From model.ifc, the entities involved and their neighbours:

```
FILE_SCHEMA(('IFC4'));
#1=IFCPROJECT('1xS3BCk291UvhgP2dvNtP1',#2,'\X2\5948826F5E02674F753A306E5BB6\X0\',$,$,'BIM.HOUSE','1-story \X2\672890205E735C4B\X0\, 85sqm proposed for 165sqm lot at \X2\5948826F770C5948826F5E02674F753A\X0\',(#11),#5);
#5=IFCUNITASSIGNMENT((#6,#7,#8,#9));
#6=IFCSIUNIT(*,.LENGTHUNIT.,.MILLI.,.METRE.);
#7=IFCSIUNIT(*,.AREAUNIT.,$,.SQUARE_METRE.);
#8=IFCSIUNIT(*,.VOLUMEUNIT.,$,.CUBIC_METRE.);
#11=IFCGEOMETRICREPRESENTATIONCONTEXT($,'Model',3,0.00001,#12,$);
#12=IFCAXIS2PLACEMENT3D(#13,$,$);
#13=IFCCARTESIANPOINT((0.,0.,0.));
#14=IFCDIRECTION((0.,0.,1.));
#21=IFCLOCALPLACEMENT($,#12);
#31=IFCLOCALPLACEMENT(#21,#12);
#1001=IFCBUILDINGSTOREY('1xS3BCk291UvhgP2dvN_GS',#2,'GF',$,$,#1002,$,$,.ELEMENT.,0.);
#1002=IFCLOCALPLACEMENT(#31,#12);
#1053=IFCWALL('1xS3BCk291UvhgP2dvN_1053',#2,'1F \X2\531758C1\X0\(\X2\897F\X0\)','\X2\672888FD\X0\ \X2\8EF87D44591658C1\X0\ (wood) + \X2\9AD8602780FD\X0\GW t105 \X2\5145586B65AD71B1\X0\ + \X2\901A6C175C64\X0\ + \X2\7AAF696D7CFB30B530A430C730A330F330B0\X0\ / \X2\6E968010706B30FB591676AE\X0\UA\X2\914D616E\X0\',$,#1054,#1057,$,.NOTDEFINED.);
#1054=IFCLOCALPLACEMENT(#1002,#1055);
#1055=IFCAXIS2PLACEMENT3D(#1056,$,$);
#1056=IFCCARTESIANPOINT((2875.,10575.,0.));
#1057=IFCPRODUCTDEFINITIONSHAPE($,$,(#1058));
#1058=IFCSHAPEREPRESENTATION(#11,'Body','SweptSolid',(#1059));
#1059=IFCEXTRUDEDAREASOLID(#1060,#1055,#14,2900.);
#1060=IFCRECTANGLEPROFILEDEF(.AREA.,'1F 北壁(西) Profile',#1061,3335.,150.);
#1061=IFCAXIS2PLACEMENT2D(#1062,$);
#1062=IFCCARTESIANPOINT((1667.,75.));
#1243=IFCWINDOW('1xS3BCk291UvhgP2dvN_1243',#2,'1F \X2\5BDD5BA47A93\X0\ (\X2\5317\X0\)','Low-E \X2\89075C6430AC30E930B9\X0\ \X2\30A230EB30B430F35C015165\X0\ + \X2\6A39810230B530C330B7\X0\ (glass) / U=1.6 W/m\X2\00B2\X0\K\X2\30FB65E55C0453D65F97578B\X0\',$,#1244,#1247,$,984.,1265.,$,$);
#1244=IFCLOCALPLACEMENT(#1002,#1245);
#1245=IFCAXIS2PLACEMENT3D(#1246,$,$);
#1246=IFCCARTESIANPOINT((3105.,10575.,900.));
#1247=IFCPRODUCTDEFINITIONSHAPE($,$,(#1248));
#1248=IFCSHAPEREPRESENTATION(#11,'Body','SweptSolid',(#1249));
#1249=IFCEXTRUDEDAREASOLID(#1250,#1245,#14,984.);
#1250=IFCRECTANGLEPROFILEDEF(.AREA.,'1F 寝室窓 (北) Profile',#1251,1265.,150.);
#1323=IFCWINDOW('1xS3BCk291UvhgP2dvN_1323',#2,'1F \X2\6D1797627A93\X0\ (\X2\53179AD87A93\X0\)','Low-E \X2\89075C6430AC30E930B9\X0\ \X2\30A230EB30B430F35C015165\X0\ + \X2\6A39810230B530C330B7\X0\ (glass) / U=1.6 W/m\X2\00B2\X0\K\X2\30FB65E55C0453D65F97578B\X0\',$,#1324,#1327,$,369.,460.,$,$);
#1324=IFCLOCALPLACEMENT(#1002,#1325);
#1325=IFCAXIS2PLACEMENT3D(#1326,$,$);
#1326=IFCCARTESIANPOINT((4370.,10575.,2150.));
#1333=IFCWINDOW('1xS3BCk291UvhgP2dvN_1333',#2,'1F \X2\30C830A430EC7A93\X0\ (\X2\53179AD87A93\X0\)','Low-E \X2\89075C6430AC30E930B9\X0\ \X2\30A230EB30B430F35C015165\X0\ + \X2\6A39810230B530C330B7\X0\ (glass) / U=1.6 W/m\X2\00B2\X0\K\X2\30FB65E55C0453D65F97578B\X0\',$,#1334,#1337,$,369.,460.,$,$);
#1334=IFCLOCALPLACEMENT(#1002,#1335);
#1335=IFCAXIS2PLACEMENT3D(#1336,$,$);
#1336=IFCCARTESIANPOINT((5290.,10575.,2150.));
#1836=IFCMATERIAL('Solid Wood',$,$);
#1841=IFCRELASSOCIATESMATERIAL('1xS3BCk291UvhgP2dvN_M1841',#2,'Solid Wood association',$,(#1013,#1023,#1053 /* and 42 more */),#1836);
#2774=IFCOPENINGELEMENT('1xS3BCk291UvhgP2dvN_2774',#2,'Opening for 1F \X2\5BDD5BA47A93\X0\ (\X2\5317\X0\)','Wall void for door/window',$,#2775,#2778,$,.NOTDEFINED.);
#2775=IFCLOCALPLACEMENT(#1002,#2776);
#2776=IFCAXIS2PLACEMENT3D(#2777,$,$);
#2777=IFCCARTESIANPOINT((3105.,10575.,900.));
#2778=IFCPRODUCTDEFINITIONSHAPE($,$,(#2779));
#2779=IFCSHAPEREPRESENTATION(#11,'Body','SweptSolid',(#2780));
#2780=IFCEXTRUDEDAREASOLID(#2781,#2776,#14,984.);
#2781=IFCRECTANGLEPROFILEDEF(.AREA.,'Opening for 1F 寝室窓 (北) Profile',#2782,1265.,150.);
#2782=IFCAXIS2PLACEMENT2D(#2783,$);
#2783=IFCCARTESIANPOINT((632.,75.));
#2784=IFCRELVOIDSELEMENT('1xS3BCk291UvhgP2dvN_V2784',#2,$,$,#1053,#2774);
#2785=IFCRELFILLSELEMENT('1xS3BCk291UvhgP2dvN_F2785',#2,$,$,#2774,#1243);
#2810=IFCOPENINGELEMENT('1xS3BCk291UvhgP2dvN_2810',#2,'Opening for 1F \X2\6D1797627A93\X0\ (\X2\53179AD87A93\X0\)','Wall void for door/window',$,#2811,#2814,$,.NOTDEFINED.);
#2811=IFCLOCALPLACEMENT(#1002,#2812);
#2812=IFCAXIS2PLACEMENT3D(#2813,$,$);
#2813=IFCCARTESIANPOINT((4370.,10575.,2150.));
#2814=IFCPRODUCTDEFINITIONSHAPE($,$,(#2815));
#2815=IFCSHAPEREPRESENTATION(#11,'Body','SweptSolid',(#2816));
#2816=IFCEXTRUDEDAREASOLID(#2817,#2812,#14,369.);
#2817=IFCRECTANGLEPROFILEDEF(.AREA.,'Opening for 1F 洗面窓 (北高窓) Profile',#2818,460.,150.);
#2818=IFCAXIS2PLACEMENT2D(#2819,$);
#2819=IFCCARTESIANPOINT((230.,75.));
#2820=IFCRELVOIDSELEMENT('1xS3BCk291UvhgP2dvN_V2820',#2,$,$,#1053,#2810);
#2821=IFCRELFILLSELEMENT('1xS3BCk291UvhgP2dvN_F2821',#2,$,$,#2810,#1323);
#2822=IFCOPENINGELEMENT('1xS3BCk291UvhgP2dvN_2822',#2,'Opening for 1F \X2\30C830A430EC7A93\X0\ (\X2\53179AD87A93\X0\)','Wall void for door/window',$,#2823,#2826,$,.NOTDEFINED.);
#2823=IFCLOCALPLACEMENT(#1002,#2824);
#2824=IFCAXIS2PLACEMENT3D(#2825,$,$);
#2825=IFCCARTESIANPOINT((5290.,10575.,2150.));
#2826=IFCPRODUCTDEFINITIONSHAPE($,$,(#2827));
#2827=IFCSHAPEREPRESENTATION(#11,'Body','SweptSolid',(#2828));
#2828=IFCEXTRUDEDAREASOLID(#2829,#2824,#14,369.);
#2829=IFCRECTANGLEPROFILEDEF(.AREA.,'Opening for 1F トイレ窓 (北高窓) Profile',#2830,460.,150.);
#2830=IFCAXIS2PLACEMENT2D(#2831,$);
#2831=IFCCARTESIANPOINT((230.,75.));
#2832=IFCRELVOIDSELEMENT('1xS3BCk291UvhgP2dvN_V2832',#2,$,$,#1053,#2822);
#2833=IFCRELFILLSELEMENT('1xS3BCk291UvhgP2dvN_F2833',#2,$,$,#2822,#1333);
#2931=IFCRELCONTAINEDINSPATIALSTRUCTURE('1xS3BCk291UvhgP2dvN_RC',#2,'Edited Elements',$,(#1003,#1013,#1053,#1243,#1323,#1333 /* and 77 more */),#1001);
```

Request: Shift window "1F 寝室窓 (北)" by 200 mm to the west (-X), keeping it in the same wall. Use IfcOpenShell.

```python
import ifcopenshell
import ifcopenshell.api.geometry
import ifcopenshell.util.placement
import ifcopenshell.util.unit

model = ifcopenshell.open("model.ifc")
unit_scale = ifcopenshell.util.unit.calculate_unit_scale(model)

window = model.by_guid("1xS3BCk291UvhgP2dvN_1243")
opening = window.FillsVoids[0].RelatingOpeningElement
wall = opening.VoidsElements[0].RelatingBuildingElement

wall_matrix = ifcopenshell.util.placement.get_local_placement(wall.ObjectPlacement)
shift = wall_matrix[:3, 0] * -0.2 / unit_scale
before = ifcopenshell.util.placement.get_local_placement(window.ObjectPlacement)[:3, 3].copy()

# The window is not placed relative to its opening, so move both.
for product in (opening, window):
    matrix = ifcopenshell.util.placement.get_local_placement(product.ObjectPlacement)
    matrix[:3, 3] += shift
    ifcopenshell.api.geometry.edit_object_placement(model, product=product, matrix=matrix, is_si=False)

after = ifcopenshell.util.placement.get_local_placement(window.ObjectPlacement)[:3, 3]
print("window moved by", (after - before).round(3) + 0.0)

model.write("model_v2.ifc")
```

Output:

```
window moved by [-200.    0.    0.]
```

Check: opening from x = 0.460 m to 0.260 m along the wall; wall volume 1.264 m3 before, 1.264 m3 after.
